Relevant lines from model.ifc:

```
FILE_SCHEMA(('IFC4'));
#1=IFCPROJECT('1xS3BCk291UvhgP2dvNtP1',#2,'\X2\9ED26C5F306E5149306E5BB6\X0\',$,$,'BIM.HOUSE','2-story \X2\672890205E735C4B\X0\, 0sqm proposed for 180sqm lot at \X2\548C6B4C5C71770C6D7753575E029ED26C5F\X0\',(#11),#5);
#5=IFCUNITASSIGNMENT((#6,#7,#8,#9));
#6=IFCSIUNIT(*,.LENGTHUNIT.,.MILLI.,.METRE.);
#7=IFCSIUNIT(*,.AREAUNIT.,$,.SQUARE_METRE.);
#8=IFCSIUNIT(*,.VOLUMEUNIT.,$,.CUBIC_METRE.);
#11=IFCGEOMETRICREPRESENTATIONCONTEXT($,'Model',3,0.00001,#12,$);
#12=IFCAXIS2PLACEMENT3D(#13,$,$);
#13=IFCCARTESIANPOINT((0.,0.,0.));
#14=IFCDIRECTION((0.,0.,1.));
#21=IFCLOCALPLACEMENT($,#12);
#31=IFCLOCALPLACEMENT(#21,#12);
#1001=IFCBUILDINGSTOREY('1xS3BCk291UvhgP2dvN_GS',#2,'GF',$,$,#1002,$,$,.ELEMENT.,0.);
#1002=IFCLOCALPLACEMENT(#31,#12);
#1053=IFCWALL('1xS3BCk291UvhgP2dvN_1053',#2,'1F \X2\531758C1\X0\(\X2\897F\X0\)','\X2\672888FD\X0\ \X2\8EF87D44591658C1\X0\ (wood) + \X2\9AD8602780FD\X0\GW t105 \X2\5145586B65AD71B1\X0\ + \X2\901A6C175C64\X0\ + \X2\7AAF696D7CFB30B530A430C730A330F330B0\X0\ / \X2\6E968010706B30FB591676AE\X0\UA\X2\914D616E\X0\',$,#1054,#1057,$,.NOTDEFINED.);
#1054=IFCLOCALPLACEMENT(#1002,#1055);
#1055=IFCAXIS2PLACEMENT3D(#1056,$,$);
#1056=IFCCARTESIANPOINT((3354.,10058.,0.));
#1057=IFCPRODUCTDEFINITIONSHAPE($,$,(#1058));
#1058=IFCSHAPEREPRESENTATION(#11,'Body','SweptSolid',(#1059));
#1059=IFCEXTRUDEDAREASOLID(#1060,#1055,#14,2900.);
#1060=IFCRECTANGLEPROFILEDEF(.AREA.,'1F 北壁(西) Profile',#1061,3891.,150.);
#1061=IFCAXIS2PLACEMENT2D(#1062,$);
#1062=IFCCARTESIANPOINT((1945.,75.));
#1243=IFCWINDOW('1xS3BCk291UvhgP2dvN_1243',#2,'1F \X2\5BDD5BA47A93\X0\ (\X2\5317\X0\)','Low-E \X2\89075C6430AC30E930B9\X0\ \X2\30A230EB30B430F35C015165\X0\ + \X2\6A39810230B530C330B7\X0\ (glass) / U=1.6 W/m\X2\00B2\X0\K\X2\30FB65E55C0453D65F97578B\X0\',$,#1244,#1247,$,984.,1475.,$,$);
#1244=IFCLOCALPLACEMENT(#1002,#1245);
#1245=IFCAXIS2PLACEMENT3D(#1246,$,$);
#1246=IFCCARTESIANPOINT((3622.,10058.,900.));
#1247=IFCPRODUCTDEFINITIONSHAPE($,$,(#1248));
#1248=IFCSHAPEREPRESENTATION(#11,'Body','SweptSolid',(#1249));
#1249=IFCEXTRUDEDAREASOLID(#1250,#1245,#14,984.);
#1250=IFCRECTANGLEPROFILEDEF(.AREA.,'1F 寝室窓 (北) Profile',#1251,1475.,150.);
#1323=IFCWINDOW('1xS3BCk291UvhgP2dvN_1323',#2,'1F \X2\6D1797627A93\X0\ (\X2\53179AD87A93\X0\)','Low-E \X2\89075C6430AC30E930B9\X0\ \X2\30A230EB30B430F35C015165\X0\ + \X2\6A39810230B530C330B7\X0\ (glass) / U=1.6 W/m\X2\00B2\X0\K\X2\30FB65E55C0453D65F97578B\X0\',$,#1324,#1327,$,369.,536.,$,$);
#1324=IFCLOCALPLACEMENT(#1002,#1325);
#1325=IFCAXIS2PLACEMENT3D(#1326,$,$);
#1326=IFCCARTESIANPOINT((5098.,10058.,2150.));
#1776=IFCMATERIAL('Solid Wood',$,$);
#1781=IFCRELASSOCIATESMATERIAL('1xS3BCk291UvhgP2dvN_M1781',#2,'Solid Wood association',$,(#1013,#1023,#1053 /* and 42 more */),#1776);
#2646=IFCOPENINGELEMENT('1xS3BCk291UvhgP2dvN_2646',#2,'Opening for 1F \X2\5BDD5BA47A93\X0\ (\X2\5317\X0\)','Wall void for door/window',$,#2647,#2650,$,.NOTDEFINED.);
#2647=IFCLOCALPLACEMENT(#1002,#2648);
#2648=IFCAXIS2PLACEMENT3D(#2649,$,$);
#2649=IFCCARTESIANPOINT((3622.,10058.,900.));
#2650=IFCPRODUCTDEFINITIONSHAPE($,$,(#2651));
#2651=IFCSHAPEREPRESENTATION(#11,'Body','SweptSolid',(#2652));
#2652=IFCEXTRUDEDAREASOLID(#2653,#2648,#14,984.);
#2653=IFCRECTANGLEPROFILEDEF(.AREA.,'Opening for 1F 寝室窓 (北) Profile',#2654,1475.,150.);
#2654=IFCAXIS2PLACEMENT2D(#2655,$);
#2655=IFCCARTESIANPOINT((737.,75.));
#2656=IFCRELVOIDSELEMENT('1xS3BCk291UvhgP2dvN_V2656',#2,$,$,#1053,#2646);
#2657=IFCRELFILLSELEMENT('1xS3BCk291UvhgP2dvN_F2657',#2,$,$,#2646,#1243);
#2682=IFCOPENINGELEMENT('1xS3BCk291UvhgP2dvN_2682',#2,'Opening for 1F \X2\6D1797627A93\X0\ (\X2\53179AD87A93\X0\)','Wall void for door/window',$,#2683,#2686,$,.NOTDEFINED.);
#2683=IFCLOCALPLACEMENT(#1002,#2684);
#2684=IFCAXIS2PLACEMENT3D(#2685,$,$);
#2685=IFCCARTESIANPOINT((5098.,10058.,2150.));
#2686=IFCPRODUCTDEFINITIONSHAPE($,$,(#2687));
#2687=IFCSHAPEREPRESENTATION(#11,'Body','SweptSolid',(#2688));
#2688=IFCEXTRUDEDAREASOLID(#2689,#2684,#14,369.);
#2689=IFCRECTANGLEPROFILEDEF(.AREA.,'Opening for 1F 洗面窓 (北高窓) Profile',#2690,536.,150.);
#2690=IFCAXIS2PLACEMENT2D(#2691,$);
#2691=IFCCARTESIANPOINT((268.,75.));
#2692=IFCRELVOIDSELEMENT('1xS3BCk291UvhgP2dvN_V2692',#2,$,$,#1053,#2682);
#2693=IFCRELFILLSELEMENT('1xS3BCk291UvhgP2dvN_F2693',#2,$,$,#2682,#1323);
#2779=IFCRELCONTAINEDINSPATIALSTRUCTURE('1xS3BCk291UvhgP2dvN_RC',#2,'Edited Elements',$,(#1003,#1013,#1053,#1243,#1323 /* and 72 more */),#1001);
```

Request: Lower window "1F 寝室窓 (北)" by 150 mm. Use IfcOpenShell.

```python
import numpy as np
import ifcopenshell
import ifcopenshell.api.geometry
import ifcopenshell.util.placement
import ifcopenshell.util.unit

model = ifcopenshell.open("model.ifc")
unit_scale = ifcopenshell.util.unit.calculate_unit_scale(model)

window = model.by_id(1243)
opening = window.FillsVoids[0].RelatingOpeningElement
dz = -150.0

shift = np.array([0.0, 0.0, dz])
# The window is not placed relative to its opening, so move both.
for product in (opening, window):
    matrix = ifcopenshell.util.placement.get_local_placement(product.ObjectPlacement)
    matrix[:3, 3] += shift
    ifcopenshell.api.geometry.edit_object_placement(model, product=product, matrix=matrix, is_si=False)

print(f"moved by {dz * unit_scale:+.3f} m")

model.write("model_rev.ifc")
```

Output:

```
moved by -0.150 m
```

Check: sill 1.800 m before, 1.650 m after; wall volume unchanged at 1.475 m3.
